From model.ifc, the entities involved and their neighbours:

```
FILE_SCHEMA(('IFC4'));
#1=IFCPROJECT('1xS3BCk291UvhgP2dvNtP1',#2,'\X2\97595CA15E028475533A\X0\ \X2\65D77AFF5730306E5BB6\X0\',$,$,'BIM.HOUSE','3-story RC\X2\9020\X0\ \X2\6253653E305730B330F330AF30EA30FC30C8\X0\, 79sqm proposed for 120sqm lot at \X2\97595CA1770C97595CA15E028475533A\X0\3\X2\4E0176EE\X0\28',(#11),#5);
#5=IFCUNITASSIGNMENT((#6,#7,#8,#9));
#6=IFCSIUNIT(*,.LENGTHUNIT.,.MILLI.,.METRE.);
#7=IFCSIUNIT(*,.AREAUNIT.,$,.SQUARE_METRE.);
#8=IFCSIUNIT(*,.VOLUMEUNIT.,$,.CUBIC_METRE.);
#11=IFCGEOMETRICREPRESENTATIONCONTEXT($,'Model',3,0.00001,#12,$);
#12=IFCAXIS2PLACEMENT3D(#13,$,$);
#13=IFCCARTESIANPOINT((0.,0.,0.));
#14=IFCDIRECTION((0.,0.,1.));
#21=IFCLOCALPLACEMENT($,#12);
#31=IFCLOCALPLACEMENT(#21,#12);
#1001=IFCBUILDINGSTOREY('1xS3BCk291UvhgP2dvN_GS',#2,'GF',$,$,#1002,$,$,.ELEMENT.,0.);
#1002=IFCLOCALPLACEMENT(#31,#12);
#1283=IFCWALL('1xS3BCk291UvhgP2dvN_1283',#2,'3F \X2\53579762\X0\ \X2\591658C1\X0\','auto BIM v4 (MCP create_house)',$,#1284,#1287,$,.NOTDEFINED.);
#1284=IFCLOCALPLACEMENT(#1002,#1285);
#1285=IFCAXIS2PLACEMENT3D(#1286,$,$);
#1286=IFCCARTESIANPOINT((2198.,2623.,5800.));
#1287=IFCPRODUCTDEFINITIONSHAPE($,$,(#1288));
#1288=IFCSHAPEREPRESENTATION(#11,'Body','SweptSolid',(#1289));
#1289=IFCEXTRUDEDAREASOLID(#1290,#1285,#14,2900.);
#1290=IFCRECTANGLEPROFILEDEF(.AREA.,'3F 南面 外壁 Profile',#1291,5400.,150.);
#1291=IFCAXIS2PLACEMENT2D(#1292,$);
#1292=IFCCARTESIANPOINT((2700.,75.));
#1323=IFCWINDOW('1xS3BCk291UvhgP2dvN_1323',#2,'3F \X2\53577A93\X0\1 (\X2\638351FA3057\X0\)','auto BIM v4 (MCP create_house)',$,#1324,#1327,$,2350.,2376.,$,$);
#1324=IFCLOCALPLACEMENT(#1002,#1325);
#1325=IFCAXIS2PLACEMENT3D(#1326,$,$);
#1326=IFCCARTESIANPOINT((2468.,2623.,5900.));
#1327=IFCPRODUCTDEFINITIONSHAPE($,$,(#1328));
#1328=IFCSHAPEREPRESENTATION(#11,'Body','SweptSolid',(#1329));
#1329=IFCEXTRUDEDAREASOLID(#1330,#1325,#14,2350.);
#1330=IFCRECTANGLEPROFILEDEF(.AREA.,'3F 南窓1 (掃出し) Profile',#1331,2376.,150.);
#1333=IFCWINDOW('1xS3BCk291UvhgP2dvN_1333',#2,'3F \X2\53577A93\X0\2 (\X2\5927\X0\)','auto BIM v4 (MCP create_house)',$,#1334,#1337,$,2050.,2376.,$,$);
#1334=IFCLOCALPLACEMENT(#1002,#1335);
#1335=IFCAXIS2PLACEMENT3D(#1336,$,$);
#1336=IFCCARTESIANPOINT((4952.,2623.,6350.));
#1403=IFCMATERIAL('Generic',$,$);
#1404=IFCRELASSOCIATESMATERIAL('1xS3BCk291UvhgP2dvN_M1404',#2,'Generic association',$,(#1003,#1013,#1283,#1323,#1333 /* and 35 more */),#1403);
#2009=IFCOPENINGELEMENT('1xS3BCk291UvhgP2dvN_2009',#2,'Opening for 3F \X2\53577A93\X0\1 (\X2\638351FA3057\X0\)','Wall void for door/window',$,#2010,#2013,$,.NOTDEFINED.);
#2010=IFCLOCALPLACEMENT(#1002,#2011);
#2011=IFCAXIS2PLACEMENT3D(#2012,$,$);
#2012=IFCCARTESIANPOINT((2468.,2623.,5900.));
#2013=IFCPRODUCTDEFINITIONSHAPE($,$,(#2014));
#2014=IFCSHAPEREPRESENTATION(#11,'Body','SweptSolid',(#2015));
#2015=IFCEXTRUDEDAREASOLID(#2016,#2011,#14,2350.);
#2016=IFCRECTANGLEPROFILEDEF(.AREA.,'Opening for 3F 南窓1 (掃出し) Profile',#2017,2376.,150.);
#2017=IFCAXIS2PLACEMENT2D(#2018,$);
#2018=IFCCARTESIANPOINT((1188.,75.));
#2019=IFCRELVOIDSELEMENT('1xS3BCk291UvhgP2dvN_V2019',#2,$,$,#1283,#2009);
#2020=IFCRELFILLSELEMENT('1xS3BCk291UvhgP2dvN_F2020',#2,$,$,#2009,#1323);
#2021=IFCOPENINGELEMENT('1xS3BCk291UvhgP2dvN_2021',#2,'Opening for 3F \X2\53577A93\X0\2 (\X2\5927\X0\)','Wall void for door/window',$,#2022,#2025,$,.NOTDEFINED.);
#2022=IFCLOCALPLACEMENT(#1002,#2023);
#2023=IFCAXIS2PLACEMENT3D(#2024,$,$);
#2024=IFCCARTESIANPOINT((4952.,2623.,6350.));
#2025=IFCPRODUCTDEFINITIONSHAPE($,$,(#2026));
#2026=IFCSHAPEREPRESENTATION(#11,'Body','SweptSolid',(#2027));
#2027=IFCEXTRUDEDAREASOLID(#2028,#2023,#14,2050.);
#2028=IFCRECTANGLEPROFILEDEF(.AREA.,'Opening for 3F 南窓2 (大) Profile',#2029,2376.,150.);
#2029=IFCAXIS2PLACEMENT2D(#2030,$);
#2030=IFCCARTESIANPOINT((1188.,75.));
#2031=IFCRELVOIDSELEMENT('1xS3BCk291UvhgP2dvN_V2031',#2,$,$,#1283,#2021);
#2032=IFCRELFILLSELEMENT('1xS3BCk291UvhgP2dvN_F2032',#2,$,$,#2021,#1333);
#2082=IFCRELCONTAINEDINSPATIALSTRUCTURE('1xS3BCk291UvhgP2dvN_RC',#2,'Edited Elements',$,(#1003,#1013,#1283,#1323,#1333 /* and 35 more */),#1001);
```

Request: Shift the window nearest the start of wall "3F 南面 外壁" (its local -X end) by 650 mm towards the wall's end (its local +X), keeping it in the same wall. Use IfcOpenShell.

```python
import ifcopenshell
import ifcopenshell.api.geometry
import ifcopenshell.util.placement
import ifcopenshell.util.unit

model = ifcopenshell.open("model.ifc")
unit_scale = ifcopenshell.util.unit.calculate_unit_scale(model)

window = model.by_guid("1xS3BCk291UvhgP2dvN_1323")
opening = window.FillsVoids[0].RelatingOpeningElement
wall = opening.VoidsElements[0].RelatingBuildingElement

wall_matrix = ifcopenshell.util.placement.get_local_placement(wall.ObjectPlacement)
shift = wall_matrix[:3, 0] * 0.65 / unit_scale
before = ifcopenshell.util.placement.get_local_placement(window.ObjectPlacement)[:3, 3].copy()

# The window is not placed relative to its opening, so move both.
for product in (opening, window):
    matrix = ifcopenshell.util.placement.get_local_placement(product.ObjectPlacement)
    matrix[:3, 3] += shift
    ifcopenshell.api.geometry.edit_object_placement(model, product=product, matrix=matrix, is_si=False)

after = ifcopenshell.util.placement.get_local_placement(window.ObjectPlacement)[:3, 3]
print("window moved by", (after - before).round(3) + 0.0)

model.write("model-out.ifc")
```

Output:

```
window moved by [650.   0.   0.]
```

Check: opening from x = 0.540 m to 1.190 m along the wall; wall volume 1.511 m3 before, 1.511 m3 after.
